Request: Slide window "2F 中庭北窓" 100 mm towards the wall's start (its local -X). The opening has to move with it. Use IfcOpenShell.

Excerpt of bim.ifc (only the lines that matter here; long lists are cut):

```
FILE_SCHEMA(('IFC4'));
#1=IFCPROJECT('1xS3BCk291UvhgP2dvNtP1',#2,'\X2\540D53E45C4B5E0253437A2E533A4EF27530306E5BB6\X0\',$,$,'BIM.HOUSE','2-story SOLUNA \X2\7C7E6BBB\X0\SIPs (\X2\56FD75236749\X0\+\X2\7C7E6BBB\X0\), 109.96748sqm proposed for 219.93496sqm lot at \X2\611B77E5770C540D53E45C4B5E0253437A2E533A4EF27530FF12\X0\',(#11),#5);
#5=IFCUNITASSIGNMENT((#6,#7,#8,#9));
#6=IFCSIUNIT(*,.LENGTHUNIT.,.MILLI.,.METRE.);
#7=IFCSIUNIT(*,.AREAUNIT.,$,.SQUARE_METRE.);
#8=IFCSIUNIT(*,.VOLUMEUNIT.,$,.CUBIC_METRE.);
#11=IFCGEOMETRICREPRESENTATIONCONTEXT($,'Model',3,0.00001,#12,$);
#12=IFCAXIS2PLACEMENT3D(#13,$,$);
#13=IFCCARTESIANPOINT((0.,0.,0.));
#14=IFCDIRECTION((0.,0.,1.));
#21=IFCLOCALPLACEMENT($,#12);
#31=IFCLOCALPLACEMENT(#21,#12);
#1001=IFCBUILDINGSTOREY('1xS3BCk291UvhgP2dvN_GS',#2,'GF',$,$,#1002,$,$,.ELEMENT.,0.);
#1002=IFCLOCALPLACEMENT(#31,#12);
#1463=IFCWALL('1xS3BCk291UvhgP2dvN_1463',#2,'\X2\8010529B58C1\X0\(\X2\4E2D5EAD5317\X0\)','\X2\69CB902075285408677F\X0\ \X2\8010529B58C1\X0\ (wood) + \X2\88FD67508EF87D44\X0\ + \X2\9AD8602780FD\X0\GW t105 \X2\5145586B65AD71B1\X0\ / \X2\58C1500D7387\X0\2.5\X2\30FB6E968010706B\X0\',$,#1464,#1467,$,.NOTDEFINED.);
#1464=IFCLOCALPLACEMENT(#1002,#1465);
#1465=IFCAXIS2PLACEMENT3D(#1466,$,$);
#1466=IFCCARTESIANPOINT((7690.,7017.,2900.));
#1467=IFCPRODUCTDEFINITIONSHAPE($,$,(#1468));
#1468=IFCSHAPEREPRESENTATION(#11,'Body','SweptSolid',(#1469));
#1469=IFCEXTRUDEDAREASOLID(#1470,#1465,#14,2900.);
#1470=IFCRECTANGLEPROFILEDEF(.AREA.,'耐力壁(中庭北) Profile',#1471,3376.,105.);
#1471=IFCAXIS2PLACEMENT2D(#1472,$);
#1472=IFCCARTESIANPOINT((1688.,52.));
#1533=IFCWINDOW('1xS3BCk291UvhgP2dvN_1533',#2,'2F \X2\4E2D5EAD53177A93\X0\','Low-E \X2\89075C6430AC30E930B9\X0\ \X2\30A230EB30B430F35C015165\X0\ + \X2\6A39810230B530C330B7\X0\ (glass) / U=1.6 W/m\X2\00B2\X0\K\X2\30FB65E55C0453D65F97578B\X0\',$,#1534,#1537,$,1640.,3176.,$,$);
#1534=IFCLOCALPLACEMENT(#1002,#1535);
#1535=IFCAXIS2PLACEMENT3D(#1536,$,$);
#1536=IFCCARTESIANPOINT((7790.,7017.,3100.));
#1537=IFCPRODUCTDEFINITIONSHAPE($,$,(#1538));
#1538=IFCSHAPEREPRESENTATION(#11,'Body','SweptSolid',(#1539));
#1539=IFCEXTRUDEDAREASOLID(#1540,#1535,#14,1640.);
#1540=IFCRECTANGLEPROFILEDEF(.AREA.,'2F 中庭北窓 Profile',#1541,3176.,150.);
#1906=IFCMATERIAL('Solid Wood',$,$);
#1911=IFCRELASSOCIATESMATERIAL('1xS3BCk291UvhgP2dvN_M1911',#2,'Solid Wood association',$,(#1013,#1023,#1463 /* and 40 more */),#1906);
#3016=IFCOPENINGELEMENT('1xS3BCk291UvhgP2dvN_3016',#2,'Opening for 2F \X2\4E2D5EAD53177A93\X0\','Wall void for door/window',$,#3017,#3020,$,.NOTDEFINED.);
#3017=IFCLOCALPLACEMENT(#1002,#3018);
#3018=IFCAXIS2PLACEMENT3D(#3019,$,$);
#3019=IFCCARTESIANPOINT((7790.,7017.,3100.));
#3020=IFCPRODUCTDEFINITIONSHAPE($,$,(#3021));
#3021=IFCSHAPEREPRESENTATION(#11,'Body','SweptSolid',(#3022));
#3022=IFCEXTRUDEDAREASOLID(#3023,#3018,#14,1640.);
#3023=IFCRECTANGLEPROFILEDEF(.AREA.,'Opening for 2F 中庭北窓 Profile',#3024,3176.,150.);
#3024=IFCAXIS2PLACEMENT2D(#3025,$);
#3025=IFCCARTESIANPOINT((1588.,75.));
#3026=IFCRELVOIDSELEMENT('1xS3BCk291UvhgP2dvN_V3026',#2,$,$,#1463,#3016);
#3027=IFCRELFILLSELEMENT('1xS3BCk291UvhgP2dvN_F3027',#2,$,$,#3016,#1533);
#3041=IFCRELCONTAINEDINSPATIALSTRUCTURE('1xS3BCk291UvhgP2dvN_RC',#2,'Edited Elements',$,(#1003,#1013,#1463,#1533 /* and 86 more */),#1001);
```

```python
import ifcopenshell
import ifcopenshell.api.geometry
import ifcopenshell.util.placement
import ifcopenshell.util.unit

model = ifcopenshell.open("bim.ifc")
unit_scale = ifcopenshell.util.unit.calculate_unit_scale(model)

window = model.by_guid("1xS3BCk291UvhgP2dvN_1533")
opening = window.FillsVoids[0].RelatingOpeningElement
wall = opening.VoidsElements[0].RelatingBuildingElement

wall_matrix = ifcopenshell.util.placement.get_local_placement(wall.ObjectPlacement)
shift = wall_matrix[:3, 0] * -0.1 / unit_scale
before = ifcopenshell.util.placement.get_local_placement(window.ObjectPlacement)[:3, 3].copy()

# The window is not placed relative to its opening, so move both.
for product in (opening, window):
    matrix = ifcopenshell.util.placement.get_local_placement(product.ObjectPlacement)
    matrix[:3, 3] += shift
    ifcopenshell.api.geometry.edit_object_placement(model, product=product, matrix=matrix, is_si=False)

after = ifcopenshell.util.placement.get_local_placement(window.ObjectPlacement)[:3, 3]
print("window moved by", (after - before).round(3) + 0.0)

model.write("bim_v2.ifc")
```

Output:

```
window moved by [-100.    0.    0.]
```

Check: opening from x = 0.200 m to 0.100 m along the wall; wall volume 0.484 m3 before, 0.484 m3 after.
